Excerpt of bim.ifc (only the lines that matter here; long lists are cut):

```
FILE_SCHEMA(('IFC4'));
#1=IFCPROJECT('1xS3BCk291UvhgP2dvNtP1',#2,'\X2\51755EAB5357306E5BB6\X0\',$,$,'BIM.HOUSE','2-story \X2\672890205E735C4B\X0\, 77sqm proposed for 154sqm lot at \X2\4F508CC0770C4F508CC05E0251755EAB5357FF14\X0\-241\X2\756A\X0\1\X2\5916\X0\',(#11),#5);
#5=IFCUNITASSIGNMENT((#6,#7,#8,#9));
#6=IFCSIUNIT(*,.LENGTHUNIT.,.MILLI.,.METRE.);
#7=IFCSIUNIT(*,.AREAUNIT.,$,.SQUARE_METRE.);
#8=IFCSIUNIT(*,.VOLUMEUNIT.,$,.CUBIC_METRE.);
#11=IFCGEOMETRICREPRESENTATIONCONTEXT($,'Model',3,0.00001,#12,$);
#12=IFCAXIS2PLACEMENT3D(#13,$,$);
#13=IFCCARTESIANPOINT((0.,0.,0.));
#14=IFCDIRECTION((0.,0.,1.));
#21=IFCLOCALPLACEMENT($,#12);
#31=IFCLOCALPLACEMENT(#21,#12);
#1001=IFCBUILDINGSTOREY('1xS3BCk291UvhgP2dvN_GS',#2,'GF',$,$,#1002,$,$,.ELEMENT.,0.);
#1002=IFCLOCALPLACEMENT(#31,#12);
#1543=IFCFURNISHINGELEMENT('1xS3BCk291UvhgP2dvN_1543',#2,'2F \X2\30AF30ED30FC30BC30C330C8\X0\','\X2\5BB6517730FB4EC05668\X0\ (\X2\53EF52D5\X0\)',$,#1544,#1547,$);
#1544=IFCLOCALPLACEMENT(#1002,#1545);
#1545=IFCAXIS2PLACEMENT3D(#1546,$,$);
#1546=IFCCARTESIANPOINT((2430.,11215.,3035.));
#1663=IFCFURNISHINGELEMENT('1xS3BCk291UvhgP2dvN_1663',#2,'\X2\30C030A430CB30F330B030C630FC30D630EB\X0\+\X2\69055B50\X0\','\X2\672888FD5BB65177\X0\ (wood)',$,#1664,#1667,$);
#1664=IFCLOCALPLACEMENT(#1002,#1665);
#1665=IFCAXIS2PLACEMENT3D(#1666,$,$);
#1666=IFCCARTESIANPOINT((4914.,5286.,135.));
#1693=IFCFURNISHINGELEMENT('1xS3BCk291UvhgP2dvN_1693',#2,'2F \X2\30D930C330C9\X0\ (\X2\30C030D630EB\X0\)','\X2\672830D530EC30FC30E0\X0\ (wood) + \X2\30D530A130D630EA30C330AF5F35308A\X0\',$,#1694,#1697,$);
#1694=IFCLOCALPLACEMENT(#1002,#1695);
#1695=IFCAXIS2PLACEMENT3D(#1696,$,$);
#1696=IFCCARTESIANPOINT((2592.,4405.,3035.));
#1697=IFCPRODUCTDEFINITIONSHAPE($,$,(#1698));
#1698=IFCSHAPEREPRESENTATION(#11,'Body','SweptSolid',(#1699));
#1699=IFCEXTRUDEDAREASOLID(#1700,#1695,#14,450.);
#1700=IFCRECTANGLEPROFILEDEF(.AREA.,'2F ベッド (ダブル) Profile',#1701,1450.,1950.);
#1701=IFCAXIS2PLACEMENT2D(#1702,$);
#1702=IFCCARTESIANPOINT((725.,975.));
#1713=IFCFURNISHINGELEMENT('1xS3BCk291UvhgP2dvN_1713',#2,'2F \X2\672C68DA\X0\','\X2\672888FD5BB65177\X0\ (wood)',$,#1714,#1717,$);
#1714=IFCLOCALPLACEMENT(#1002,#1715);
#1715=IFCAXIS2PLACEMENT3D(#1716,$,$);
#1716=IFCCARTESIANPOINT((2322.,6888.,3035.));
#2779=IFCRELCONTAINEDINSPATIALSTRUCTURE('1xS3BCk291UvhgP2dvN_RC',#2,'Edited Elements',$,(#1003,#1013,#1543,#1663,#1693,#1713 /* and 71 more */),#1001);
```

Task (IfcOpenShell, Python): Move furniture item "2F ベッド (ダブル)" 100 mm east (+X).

```python
import ifcopenshell
import ifcopenshell.api.geometry
import ifcopenshell.util.placement
import ifcopenshell.util.unit

model = ifcopenshell.open("bim.ifc")
unit_scale = ifcopenshell.util.unit.calculate_unit_scale(model)

item = model.by_id(1693)
matrix = ifcopenshell.util.placement.get_local_placement(item.ObjectPlacement)
matrix[0, 3] += 0.1 / unit_scale
ifcopenshell.api.geometry.edit_object_placement(model, product=item, matrix=matrix, is_si=False)

print(ifcopenshell.util.placement.get_local_placement(item.ObjectPlacement).round(3) + 0.0)

model.write("bim_edited.ifc")
```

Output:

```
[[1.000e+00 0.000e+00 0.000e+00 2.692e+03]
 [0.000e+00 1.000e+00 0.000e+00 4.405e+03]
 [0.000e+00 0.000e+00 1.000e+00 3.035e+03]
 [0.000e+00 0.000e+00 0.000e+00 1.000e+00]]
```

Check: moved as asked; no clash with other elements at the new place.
